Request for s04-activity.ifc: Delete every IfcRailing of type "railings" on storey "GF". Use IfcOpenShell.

First a look at what the model holds.

```python
import ifcopenshell
import ifcopenshell.util.element

model = ifcopenshell.open("s04-activity.ifc")
print(model.schema)
storey = next(s for s in model.by_type("IfcBuildingStorey") if s.Name == "GF")
railings = [e for e in ifcopenshell.util.element.get_decomposition(storey) if e.is_a("IfcRailing")]
seen = {}
for e in railings:
    element_type = ifcopenshell.util.element.get_type(e)
    name = element_type.Name if element_type not in (None, e) else None
    seen[name] = seen.get(name, 0) + 1
for name, count in sorted(seen.items(), key=str):
    print(count, "x", name)
```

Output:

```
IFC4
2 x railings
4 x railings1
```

```python
import ifcopenshell
import ifcopenshell.api.root
import ifcopenshell.util.element

model = ifcopenshell.open("s04-activity.ifc")

storey = next(s for s in model.by_type("IfcBuildingStorey") if s.Name == "GF")
railings = [e for e in ifcopenshell.util.element.get_decomposition(storey) if e.is_a("IfcRailing")]
targets = [e for e in railings if (t := ifcopenshell.util.element.get_type(e)) not in (None, e) and t.Name == "railings"]

for e in targets:
    ifcopenshell.api.root.remove_product(model, product=e)
print(len(targets), "removed")

model.write("s04-activity_updated.ifc")
```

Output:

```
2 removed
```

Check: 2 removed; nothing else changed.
